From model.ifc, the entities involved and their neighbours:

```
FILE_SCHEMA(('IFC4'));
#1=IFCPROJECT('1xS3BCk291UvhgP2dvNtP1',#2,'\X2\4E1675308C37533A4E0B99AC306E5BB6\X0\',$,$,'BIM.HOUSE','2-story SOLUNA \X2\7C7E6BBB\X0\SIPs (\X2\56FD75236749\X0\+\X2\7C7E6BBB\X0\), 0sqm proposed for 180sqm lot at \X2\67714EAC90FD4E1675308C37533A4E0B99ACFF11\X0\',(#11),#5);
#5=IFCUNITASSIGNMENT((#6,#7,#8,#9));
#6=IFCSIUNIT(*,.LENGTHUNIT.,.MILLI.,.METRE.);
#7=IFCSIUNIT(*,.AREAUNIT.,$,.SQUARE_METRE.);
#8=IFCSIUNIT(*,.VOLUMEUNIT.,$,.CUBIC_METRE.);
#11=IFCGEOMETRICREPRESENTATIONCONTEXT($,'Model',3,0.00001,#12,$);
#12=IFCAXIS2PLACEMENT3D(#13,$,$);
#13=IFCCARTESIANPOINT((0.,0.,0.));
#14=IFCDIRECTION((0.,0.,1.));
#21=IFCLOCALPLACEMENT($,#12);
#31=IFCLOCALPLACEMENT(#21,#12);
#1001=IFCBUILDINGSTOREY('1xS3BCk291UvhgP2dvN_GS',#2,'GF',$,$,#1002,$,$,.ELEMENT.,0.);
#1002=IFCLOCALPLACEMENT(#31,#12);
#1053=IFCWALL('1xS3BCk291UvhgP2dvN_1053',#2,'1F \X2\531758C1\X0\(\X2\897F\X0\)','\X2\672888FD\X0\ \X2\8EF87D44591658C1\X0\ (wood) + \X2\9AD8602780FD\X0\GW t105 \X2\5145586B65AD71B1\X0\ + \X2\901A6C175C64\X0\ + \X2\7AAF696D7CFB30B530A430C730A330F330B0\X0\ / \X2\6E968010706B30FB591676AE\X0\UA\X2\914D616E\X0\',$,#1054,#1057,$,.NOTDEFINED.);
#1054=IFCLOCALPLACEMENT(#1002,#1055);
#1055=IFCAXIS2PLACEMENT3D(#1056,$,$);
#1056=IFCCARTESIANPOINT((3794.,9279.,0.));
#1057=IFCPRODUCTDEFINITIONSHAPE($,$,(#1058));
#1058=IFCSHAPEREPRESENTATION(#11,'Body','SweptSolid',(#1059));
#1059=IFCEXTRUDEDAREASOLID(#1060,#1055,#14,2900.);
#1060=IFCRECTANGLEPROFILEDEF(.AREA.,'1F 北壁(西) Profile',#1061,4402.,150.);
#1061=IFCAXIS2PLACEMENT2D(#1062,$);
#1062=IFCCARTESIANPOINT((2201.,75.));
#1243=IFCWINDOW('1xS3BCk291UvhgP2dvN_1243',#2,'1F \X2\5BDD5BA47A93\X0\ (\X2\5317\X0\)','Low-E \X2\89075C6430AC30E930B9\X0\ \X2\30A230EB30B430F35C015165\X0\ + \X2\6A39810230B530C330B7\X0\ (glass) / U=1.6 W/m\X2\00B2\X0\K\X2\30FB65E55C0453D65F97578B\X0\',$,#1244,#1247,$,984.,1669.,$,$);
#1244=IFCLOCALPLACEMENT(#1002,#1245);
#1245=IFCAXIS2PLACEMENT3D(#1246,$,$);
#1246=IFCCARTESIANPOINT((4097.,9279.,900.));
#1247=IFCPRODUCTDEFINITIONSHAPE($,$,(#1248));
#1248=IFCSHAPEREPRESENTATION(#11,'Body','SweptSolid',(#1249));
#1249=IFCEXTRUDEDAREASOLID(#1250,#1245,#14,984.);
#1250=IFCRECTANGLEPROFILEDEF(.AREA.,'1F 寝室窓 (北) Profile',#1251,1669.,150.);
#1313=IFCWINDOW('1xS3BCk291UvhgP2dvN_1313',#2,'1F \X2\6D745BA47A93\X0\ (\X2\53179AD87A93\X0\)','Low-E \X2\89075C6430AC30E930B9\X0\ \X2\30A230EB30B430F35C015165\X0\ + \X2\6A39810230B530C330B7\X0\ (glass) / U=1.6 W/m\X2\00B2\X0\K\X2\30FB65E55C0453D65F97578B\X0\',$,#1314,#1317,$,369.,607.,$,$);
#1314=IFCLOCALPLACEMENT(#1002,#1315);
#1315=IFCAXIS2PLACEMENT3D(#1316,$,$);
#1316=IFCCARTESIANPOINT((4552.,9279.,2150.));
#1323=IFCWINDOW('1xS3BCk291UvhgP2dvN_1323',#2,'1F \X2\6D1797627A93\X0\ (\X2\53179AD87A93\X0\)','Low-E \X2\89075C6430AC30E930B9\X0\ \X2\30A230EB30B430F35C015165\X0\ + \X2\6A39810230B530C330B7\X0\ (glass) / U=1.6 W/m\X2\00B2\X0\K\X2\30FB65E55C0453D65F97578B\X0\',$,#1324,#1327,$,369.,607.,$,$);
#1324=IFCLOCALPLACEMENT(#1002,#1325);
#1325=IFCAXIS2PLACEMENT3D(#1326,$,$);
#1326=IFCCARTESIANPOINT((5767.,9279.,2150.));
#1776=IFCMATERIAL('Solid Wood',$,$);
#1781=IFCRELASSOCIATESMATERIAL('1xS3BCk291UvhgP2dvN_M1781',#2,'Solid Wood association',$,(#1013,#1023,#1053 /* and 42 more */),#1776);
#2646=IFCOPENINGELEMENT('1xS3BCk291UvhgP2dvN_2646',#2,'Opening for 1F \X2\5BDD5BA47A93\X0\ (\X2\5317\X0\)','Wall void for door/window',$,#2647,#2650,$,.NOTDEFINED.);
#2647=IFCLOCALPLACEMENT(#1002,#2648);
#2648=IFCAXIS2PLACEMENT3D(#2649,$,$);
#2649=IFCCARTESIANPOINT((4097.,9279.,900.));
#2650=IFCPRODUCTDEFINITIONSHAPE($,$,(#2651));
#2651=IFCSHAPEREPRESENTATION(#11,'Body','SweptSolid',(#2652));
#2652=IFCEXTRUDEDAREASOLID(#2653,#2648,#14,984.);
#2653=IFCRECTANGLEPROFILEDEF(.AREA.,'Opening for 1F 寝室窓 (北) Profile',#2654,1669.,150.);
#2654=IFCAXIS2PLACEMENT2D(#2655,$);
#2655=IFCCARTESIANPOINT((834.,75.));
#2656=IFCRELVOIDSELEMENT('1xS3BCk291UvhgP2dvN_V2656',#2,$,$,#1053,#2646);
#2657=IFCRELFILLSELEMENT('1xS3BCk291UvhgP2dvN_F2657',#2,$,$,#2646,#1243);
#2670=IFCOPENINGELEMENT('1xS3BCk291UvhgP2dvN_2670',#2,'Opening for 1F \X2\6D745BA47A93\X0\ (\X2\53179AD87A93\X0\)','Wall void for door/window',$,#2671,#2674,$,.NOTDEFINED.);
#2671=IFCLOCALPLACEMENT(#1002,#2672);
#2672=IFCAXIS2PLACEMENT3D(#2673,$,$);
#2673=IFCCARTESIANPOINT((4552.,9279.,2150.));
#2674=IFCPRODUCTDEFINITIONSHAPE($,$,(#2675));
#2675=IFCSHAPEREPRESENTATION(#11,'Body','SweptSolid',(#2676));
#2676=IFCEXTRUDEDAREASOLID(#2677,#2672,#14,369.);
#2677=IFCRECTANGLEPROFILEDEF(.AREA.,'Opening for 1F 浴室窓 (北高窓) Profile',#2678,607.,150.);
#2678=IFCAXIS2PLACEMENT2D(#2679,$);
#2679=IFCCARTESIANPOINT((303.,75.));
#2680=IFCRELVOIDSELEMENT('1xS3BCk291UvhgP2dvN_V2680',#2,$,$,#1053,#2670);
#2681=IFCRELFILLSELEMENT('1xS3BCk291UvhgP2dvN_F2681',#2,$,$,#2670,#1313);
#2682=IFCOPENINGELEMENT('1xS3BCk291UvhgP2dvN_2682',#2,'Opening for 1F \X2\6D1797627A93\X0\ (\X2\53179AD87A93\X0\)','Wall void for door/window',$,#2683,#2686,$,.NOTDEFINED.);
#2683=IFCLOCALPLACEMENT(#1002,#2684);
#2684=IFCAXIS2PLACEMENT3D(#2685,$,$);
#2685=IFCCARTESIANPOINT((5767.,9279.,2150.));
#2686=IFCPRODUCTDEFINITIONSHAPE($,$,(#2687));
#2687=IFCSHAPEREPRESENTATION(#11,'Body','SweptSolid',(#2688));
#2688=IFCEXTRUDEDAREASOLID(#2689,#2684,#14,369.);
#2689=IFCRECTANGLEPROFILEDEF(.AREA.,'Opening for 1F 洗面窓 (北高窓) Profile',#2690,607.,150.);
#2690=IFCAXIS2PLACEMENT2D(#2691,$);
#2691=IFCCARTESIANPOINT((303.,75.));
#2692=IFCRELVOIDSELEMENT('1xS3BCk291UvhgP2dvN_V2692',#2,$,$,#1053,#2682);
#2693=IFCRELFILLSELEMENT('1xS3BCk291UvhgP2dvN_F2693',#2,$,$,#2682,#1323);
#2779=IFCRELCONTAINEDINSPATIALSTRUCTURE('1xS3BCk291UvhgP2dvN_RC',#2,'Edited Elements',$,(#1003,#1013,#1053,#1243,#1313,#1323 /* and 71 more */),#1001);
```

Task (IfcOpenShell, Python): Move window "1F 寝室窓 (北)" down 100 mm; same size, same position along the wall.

```python
import numpy as np
import ifcopenshell
import ifcopenshell.api.geometry
import ifcopenshell.util.placement
import ifcopenshell.util.unit

model = ifcopenshell.open("model.ifc")
unit_scale = ifcopenshell.util.unit.calculate_unit_scale(model)

window = model.by_guid("1xS3BCk291UvhgP2dvN_1243")
opening = window.FillsVoids[0].RelatingOpeningElement
dz = -100.0

shift = np.array([0.0, 0.0, dz])
# The window is not placed relative to its opening, so move both.
for product in (opening, window):
    matrix = ifcopenshell.util.placement.get_local_placement(product.ObjectPlacement)
    matrix[:3, 3] += shift
    ifcopenshell.api.geometry.edit_object_placement(model, product=product, matrix=matrix, is_si=False)

print(f"moved by {dz * unit_scale:+.3f} m")

model.write("model_v2.ifc")
```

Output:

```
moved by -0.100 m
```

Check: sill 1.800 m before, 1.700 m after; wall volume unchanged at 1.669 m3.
